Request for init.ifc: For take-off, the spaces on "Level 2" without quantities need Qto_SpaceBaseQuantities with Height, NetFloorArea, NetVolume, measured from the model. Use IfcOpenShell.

First a look at what the model holds.

```python
import ifcopenshell
import ifcopenshell.util.element
import ifcopenshell.util.unit

model = ifcopenshell.open("init.ifc")
print(model.schema)
for unit_type in ("LENGTHUNIT", "AREAUNIT", "VOLUMEUNIT"):
    print(unit_type, ifcopenshell.util.unit.calculate_unit_scale(model, unit_type))
storey = next(s for s in model.by_type("IfcBuildingStorey") if s.Name == "Level 2")
spaces = [e for e in ifcopenshell.util.element.get_decomposition(storey) if e.is_a("IfcSpace")]
for e in sorted(spaces, key=lambda e: e.id()):
    print(e.id(), e.is_a(), e.Name, list(ifcopenshell.util.element.get_psets(e, qtos_only=True)), sep=" | ")
```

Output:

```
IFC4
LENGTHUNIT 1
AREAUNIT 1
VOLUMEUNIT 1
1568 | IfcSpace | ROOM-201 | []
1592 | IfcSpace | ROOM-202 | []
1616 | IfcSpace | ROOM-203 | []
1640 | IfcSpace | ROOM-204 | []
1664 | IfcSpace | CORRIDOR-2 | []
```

```python
import ifcopenshell
import ifcopenshell.api.pset
import ifcopenshell.geom
import ifcopenshell.util.element
import ifcopenshell.util.shape
import ifcopenshell.util.unit

model = ifcopenshell.open("init.ifc")
unit_scale = ifcopenshell.util.unit.calculate_unit_scale(model)
area_scale = ifcopenshell.util.unit.calculate_unit_scale(model, "AREAUNIT")
volume_scale = ifcopenshell.util.unit.calculate_unit_scale(model, "VOLUMEUNIT")
settings = ifcopenshell.geom.settings()

storey = next(s for s in model.by_type("IfcBuildingStorey") if s.Name == "Level 2")
spaces = [e for e in ifcopenshell.util.element.get_decomposition(storey) if e.is_a("IfcSpace")]

for e in sorted(spaces, key=lambda e: e.id()):
    if ifcopenshell.util.element.get_psets(e, qtos_only=True, should_inherit=False):
        continue
    # Geometry comes back in metres, in the element's own axes.
    shape = ifcopenshell.geom.create_shape(settings, e)
    values = {
        "Height": ifcopenshell.util.shape.get_z(shape.geometry) / unit_scale,
        "NetFloorArea": ifcopenshell.util.shape.get_footprint_area(shape.geometry) / area_scale,
        "NetVolume": ifcopenshell.util.shape.get_volume(shape.geometry) / volume_scale,
    }
    qto = ifcopenshell.api.pset.add_qto(model, product=e, name="Qto_SpaceBaseQuantities")
    ifcopenshell.api.pset.edit_qto(model, qto=qto, properties=values)
    print(e.id(), {k: round(v, 3) for k, v in values.items()})

model.write("init_updated.ifc")
```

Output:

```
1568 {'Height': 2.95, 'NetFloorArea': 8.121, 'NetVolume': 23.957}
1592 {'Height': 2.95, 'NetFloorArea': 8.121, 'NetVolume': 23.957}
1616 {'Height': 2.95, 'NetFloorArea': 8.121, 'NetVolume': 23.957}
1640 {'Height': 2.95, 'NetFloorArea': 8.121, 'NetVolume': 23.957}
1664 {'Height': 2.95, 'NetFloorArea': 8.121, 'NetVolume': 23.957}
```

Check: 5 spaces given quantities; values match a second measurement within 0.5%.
